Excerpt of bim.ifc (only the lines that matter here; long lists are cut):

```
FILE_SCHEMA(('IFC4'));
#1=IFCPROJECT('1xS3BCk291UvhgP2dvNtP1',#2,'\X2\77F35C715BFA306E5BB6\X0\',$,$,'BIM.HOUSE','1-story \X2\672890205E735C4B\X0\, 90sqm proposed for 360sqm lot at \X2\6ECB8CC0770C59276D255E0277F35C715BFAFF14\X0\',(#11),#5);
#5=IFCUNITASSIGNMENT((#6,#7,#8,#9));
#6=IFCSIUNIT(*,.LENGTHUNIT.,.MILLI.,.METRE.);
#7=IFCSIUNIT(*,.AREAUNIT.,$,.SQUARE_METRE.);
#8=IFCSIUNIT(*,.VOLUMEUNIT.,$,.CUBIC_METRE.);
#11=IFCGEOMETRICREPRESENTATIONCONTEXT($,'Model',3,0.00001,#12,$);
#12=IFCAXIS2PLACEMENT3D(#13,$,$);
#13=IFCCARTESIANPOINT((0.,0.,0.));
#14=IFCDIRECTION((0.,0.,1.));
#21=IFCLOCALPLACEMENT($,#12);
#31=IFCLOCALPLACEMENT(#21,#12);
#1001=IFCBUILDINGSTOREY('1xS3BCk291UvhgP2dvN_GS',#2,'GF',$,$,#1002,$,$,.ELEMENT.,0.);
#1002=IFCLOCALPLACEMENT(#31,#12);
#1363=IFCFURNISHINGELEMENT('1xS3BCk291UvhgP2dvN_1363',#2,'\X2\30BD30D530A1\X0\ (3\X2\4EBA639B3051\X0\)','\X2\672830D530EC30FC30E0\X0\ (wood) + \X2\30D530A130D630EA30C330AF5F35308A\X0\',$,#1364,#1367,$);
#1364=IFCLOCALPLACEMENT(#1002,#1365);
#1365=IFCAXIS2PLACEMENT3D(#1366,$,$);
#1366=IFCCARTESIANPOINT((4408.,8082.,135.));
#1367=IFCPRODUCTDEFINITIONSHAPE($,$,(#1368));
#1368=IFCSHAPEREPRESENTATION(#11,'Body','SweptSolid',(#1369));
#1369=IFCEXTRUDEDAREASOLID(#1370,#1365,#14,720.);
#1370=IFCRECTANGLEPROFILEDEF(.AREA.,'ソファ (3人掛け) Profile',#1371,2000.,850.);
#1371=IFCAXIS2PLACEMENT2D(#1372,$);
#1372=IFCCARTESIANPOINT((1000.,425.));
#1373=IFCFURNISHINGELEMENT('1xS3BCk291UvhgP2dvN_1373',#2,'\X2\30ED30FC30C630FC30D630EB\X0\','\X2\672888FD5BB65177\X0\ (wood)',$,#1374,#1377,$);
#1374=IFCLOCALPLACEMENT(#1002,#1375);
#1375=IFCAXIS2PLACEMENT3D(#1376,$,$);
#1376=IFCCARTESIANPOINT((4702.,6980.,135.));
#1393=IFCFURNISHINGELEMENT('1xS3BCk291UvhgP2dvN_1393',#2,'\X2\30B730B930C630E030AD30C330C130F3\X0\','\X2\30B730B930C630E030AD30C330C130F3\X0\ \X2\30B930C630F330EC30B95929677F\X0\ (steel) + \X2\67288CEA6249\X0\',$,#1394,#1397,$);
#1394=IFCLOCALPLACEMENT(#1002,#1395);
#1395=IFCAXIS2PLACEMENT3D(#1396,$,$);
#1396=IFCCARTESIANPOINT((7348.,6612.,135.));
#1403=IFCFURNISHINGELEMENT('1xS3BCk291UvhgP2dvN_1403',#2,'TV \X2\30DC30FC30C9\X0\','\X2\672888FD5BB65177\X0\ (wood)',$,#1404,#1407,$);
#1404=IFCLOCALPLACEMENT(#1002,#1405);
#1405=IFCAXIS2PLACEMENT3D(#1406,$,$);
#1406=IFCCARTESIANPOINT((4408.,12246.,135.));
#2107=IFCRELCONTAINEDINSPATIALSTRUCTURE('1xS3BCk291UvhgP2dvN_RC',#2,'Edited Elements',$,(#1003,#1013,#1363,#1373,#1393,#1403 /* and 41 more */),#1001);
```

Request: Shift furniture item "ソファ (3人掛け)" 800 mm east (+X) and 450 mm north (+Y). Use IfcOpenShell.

```python
import ifcopenshell
import ifcopenshell.api.geometry
import ifcopenshell.util.placement

model = ifcopenshell.open("bim.ifc")

item = model.by_id(1363)
matrix = ifcopenshell.util.placement.get_local_placement(item.ObjectPlacement)
matrix[0, 3] += 800.0
matrix[1, 3] += 450.0
ifcopenshell.api.geometry.edit_object_placement(model, product=item, matrix=matrix, is_si=False)

print(ifcopenshell.util.placement.get_local_placement(item.ObjectPlacement).round(3) + 0.0)

model.write("bim_edited.ifc")
```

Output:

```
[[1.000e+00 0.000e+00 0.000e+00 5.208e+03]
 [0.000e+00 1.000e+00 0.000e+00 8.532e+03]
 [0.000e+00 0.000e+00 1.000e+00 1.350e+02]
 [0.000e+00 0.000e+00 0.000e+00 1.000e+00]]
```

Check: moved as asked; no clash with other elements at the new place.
